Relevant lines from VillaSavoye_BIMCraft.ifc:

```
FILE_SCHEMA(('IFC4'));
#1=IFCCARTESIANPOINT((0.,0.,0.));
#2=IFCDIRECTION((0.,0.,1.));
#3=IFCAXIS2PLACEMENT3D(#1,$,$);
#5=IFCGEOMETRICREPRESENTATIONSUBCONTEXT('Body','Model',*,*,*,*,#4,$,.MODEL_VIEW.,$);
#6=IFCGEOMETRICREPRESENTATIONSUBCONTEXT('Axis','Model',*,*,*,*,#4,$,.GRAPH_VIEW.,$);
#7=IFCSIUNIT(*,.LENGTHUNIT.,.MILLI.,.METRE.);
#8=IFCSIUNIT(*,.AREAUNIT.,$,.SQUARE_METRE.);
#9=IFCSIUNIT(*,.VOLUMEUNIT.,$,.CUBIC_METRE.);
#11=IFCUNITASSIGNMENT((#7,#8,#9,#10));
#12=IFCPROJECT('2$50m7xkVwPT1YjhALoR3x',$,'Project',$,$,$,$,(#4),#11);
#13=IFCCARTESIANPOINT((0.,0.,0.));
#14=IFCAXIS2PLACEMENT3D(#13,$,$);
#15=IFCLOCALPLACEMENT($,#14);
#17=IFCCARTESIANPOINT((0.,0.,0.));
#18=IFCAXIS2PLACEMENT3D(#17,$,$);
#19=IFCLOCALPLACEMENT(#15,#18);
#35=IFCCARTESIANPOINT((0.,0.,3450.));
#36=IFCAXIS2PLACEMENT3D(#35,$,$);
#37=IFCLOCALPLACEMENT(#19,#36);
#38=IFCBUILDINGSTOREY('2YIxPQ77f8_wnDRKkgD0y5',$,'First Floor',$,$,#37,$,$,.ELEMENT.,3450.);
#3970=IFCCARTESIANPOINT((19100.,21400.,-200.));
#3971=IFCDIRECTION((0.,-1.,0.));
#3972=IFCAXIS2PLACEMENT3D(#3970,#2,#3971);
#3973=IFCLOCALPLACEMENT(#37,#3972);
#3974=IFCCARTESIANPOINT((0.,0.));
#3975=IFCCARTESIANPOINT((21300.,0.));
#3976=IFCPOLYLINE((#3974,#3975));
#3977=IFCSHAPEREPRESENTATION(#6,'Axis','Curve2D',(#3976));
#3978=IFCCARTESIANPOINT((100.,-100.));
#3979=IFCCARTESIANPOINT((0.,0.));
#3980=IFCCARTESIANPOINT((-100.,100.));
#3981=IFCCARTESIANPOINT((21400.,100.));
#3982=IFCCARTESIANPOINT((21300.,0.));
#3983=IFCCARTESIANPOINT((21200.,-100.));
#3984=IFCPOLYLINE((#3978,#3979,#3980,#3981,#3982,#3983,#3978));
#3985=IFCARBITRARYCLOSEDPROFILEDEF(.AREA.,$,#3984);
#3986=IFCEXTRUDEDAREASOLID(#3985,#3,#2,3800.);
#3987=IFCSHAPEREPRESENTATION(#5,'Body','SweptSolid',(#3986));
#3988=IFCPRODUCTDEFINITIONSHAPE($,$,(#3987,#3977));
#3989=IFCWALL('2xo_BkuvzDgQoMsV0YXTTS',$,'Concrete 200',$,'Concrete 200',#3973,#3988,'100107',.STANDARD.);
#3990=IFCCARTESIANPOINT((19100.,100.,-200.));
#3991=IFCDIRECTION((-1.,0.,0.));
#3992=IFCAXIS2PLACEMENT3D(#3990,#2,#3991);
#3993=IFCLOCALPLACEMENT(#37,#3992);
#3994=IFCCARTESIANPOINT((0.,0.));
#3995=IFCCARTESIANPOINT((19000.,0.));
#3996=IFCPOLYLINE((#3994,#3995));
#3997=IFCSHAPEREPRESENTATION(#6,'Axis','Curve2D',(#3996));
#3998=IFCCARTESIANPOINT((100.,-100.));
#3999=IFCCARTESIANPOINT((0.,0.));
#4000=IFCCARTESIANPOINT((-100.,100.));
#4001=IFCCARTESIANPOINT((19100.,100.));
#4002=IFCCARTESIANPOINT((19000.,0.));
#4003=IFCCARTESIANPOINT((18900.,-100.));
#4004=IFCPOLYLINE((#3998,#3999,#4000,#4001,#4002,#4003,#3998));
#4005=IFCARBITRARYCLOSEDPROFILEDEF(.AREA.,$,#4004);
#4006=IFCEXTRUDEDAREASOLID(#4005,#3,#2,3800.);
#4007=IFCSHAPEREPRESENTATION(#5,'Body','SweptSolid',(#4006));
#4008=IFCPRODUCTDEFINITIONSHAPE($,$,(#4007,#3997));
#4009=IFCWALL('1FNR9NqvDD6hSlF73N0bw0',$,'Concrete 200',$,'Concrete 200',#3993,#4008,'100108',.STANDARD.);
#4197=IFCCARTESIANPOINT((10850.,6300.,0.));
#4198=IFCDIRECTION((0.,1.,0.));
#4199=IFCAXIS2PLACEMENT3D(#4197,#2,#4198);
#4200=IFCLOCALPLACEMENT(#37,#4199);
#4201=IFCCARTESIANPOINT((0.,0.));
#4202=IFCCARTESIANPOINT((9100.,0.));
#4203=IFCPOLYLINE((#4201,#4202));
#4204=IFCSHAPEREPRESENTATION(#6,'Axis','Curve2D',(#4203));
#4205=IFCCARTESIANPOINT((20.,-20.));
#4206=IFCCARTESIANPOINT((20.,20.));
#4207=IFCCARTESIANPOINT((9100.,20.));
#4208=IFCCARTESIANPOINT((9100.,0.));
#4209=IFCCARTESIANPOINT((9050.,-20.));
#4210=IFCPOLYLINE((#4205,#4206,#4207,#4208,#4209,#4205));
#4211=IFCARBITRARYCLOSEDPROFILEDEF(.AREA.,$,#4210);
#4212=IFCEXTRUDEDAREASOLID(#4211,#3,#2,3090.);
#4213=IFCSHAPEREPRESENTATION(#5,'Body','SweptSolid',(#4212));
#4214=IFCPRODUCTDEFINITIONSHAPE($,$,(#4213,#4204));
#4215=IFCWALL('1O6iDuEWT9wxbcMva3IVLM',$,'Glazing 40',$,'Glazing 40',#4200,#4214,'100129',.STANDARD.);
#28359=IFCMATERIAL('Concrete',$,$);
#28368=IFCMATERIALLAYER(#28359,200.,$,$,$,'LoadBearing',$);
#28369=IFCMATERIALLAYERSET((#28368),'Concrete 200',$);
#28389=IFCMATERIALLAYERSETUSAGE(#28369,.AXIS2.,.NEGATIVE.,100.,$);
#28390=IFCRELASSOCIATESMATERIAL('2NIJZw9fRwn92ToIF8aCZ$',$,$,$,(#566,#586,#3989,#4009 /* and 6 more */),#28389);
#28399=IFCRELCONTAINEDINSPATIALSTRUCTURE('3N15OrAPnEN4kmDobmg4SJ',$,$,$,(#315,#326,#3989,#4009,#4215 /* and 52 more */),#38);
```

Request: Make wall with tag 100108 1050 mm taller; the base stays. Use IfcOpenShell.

```python
import ifcopenshell
import ifcopenshell.geom
import ifcopenshell.util.representation
import ifcopenshell.util.shape
import ifcopenshell.util.unit

model = ifcopenshell.open("VillaSavoye_BIMCraft.ifc")
unit_scale = ifcopenshell.util.unit.calculate_unit_scale(model)
settings = ifcopenshell.geom.settings()


def volume(element):
    """Net volume in cubic metres, openings subtracted."""
    shape = ifcopenshell.geom.create_shape(settings, element)
    return ifcopenshell.util.shape.get_volume(shape.geometry)


wall = model.by_guid("1FNR9NqvDD6hSlF73N0bw0")
before = volume(wall)

body = ifcopenshell.util.representation.get_representation(wall, "Model", "Body")
solid = body.Items[0]
old_height = solid.Depth
solid.Depth += 1.05 / unit_scale
after = volume(wall)

print(f"height {old_height:g} -> {solid.Depth:g}, volume {before:.3f} -> {after:.3f} m3")

model.write("VillaSavoye_BIMCraft_rev.ifc")
```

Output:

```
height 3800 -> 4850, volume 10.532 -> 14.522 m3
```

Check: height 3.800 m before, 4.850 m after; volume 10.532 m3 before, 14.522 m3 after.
